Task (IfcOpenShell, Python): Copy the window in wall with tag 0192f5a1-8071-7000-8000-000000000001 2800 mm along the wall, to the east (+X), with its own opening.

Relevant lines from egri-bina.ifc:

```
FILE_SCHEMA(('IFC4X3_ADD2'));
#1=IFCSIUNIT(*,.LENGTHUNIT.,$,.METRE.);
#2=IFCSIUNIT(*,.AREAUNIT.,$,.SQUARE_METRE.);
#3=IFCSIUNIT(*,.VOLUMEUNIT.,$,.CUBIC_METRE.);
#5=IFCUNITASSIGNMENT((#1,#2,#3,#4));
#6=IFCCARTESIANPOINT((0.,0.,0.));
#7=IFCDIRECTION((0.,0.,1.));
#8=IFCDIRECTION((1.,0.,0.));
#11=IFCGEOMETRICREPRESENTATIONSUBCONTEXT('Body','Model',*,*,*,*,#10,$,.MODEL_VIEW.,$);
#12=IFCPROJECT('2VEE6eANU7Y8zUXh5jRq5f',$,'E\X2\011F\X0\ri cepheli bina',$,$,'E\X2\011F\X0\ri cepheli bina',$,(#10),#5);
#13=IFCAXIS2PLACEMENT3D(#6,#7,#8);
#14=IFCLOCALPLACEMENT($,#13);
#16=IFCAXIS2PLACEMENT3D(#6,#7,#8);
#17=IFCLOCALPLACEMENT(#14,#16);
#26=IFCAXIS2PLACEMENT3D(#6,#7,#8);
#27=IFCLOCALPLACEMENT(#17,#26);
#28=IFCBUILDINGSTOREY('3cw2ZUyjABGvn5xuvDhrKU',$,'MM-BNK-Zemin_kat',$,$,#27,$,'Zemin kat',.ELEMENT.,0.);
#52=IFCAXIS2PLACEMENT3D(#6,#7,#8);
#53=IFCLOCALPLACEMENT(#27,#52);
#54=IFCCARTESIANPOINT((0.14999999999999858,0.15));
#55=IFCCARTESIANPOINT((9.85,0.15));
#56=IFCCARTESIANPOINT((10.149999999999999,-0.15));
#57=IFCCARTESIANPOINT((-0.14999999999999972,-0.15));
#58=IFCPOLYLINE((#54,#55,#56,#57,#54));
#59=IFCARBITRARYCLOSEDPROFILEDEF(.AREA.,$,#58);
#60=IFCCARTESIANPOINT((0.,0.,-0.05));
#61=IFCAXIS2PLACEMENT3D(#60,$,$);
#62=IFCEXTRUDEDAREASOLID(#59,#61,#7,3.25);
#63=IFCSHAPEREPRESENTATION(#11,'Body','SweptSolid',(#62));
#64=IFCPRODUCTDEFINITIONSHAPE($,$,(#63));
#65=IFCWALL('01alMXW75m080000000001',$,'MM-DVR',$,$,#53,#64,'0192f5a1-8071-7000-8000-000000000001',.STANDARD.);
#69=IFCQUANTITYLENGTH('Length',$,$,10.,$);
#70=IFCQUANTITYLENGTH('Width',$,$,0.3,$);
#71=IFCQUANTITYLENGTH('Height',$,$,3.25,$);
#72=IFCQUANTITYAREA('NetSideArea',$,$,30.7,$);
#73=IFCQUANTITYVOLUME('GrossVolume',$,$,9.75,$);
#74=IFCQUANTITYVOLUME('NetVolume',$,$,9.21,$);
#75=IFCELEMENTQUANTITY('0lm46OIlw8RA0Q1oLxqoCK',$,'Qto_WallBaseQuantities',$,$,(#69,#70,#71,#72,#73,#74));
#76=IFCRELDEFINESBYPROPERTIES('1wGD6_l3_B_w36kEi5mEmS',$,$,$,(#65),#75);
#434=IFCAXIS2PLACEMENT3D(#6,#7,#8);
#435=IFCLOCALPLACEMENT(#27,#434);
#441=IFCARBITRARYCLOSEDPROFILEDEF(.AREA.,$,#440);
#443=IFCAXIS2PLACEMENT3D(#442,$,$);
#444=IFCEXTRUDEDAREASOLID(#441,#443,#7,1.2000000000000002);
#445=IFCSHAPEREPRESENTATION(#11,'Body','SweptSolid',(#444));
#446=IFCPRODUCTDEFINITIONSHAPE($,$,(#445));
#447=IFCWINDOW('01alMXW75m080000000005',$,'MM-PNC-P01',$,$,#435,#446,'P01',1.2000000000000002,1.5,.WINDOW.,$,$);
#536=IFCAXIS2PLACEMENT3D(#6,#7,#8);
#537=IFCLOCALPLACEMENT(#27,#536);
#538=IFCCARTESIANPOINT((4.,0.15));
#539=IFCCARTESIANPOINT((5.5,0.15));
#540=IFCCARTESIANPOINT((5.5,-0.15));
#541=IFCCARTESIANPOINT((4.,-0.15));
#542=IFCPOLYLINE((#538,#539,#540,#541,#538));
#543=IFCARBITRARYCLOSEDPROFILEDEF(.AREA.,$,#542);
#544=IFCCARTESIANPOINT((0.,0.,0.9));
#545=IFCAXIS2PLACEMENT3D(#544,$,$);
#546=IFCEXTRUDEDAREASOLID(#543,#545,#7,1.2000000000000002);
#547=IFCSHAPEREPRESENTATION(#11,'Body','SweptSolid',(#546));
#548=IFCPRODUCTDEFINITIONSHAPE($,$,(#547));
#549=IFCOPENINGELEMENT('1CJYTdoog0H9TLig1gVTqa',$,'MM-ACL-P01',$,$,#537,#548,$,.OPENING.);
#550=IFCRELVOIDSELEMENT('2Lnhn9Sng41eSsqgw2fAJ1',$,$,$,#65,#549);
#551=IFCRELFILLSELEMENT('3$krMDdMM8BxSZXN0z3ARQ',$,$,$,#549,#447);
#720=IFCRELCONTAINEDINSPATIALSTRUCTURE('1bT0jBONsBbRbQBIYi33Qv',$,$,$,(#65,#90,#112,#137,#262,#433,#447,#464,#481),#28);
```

```python
import ifcopenshell
import ifcopenshell.api.feature
import ifcopenshell.api.geometry
import ifcopenshell.api.pset
import ifcopenshell.api.root
import ifcopenshell.geom
import ifcopenshell.util.element
import ifcopenshell.util.placement
import ifcopenshell.util.shape
import ifcopenshell.util.unit

model = ifcopenshell.open("egri-bina.ifc")
area_scale = ifcopenshell.util.unit.calculate_unit_scale(model, "AREAUNIT")
volume_scale = ifcopenshell.util.unit.calculate_unit_scale(model, "VOLUMEUNIT")
settings = ifcopenshell.geom.settings()


def volume(element):
    """Net volume in cubic metres, openings subtracted."""
    shape = ifcopenshell.geom.create_shape(settings, element)
    return ifcopenshell.util.shape.get_volume(shape.geometry)


window = model.by_guid("01alMXW75m080000000005")
opening = window.FillsVoids[0].RelatingOpeningElement
wall = opening.VoidsElements[0].RelatingBuildingElement
before = volume(wall)
shift = ifcopenshell.util.placement.get_local_placement(wall.ObjectPlacement)[:3, 0] * 2.8

# copy_class copies the void relationship, type, container and properties, but no geometry.
new_opening = ifcopenshell.api.root.copy_class(model, product=opening)
new_opening.Representation = ifcopenshell.util.element.copy_deep(
    model, opening.Representation, exclude=["IfcGeometricRepresentationContext", "IfcRepresentationMap"]
)
new_window = ifcopenshell.api.root.copy_class(model, product=window)
new_window.Representation = ifcopenshell.util.element.copy_deep(
    model, window.Representation, exclude=["IfcGeometricRepresentationContext", "IfcRepresentationMap"]
)
new_window.Tag = None
ifcopenshell.api.feature.add_filling(model, opening=new_opening, element=new_window)

for old, new in ((opening, new_opening), (window, new_window)):
    matrix = ifcopenshell.util.placement.get_local_placement(old.ObjectPlacement)
    matrix[:3, 3] += shift
    ifcopenshell.api.geometry.edit_object_placement(model, product=new, matrix=matrix, is_si=False)

after = volume(wall)
thickness = 0.3  # wall thickness in metres

# Update the wall's stored quantities.
qto = model.by_id(ifcopenshell.util.element.get_pset(wall, "Qto_WallBaseQuantities", should_inherit=False)["id"])
ifcopenshell.api.pset.edit_qto(model, qto=qto, properties={
    "NetSideArea": after / thickness / area_scale,
    "NetVolume": after / volume_scale,
})

print(f"wall volume {before:.3f} -> {after:.3f} m3")

model.write("egri-bina_v2.ifc")
```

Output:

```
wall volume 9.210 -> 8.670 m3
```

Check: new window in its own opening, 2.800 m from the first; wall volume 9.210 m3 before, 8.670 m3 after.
